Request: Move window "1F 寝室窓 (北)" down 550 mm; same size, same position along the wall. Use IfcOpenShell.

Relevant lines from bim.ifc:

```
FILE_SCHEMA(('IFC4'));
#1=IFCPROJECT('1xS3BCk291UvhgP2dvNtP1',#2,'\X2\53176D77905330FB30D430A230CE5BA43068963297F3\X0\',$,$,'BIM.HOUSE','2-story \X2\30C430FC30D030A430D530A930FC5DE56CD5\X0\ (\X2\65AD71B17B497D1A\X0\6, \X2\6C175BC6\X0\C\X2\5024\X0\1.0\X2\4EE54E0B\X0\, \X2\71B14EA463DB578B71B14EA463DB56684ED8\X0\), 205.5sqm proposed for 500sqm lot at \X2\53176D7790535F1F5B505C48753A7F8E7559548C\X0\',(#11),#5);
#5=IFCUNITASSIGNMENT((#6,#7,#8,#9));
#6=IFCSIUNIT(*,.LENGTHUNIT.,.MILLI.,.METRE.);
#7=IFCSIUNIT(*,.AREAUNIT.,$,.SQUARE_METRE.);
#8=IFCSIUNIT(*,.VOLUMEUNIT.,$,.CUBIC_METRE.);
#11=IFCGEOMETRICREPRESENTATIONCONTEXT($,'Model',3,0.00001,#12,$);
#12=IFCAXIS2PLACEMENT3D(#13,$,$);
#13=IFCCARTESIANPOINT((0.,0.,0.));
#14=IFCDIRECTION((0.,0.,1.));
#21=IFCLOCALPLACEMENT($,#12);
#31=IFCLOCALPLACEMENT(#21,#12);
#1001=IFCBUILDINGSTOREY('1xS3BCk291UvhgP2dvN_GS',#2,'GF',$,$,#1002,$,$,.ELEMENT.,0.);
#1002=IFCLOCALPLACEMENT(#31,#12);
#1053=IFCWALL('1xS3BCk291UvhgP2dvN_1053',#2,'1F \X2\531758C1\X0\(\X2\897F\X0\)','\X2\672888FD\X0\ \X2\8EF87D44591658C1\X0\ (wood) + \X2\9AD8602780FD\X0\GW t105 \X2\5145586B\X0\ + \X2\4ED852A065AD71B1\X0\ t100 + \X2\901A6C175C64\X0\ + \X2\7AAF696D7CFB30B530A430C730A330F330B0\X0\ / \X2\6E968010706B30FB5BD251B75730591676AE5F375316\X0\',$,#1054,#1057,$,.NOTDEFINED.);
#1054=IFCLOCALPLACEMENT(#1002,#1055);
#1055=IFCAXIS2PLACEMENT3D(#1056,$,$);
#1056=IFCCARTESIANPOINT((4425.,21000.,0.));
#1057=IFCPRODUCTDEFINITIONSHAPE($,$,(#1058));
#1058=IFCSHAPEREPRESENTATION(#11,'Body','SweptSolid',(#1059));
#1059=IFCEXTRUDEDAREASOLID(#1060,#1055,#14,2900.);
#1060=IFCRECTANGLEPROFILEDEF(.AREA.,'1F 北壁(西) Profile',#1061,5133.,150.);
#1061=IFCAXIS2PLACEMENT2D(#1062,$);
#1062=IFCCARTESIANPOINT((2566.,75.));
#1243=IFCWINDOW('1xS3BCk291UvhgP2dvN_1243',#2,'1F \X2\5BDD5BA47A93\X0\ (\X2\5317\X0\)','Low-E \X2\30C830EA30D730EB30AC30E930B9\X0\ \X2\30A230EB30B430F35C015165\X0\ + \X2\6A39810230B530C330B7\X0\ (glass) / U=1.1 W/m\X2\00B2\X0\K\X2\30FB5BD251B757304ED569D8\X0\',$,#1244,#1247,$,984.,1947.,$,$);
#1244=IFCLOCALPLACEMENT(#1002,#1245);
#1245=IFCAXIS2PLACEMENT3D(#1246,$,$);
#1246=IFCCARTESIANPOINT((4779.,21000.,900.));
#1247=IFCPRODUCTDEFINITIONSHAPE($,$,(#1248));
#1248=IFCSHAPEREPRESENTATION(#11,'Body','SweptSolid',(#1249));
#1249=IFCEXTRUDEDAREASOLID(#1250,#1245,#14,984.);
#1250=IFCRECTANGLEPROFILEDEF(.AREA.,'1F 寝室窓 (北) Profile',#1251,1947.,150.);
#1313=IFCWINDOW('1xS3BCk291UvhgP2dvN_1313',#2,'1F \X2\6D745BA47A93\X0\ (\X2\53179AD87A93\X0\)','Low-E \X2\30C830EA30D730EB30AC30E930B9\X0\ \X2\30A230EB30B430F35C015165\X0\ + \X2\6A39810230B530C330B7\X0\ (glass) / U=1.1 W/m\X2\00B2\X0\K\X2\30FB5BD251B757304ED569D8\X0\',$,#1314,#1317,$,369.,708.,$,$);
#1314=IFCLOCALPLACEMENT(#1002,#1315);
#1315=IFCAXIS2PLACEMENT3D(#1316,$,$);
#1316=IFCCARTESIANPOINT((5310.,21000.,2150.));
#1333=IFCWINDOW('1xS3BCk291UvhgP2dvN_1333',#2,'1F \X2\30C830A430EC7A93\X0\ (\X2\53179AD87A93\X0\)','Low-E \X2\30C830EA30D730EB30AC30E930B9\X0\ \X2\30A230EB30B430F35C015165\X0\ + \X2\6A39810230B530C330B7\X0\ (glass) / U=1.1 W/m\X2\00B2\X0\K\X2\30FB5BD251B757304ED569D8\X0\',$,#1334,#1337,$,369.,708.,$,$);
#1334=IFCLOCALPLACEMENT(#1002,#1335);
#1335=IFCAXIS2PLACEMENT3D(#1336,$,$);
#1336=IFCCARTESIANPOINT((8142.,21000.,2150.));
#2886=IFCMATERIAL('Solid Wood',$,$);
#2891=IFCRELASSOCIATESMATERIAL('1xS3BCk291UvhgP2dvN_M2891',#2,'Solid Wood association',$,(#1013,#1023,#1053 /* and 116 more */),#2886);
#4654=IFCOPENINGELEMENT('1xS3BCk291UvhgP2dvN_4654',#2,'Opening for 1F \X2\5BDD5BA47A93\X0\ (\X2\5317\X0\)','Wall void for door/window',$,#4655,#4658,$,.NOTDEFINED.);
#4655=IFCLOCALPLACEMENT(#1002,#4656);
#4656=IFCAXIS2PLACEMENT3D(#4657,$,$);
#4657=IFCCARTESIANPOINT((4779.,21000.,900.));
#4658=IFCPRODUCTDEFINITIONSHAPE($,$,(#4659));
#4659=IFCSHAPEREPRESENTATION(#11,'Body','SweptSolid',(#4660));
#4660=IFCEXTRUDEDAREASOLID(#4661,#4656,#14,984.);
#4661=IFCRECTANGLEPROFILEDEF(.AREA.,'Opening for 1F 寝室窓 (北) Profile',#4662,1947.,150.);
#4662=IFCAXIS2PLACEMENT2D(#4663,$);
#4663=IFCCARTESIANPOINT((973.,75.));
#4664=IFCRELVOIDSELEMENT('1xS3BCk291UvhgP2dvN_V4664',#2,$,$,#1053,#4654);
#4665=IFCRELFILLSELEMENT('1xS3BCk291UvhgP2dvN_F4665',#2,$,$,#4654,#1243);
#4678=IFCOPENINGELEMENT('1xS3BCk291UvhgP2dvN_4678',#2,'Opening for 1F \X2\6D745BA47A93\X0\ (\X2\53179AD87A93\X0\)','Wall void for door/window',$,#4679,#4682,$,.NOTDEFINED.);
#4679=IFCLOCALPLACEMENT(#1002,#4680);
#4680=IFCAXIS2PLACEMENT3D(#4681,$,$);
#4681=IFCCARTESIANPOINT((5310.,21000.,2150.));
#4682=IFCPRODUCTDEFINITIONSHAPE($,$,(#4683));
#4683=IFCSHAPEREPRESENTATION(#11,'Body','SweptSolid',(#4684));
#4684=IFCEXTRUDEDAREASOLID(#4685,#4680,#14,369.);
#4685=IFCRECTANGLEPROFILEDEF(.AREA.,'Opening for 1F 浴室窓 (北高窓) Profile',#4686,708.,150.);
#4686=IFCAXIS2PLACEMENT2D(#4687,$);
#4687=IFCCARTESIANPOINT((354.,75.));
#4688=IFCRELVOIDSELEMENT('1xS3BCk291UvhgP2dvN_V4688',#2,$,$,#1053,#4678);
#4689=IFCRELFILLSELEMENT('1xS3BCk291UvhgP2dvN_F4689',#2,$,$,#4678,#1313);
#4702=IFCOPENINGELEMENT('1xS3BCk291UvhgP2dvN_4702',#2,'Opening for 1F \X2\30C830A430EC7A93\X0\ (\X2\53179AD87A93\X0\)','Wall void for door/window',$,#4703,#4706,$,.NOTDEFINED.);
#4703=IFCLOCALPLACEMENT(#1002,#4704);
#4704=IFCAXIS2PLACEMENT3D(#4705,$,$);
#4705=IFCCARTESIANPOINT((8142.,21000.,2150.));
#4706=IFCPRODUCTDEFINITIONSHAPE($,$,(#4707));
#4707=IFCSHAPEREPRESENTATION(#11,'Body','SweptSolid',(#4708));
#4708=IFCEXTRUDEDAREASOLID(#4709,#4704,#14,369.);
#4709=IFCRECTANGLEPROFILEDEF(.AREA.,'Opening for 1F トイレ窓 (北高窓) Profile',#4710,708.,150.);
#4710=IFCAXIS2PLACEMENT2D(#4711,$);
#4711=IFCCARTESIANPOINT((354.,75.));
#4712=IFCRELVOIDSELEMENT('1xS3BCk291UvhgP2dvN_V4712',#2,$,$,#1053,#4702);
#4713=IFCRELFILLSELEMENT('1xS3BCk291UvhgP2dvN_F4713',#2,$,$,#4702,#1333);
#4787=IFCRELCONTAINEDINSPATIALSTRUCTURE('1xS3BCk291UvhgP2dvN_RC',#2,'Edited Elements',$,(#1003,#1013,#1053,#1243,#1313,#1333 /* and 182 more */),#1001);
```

```python
import numpy as np
import ifcopenshell
import ifcopenshell.api.geometry
import ifcopenshell.util.placement
import ifcopenshell.util.unit

model = ifcopenshell.open("bim.ifc")
unit_scale = ifcopenshell.util.unit.calculate_unit_scale(model)

window = model.by_id(1243)
opening = window.FillsVoids[0].RelatingOpeningElement
dz = -0.55 / unit_scale

shift = np.array([0.0, 0.0, dz])
# The window is not placed relative to its opening, so move both.
for product in (opening, window):
    matrix = ifcopenshell.util.placement.get_local_placement(product.ObjectPlacement)
    matrix[:3, 3] += shift
    ifcopenshell.api.geometry.edit_object_placement(model, product=product, matrix=matrix, is_si=False)

print(f"moved by {dz * unit_scale:+.3f} m")

model.write("bim_edited.ifc")
```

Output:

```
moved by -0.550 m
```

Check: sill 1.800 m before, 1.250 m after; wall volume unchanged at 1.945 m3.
